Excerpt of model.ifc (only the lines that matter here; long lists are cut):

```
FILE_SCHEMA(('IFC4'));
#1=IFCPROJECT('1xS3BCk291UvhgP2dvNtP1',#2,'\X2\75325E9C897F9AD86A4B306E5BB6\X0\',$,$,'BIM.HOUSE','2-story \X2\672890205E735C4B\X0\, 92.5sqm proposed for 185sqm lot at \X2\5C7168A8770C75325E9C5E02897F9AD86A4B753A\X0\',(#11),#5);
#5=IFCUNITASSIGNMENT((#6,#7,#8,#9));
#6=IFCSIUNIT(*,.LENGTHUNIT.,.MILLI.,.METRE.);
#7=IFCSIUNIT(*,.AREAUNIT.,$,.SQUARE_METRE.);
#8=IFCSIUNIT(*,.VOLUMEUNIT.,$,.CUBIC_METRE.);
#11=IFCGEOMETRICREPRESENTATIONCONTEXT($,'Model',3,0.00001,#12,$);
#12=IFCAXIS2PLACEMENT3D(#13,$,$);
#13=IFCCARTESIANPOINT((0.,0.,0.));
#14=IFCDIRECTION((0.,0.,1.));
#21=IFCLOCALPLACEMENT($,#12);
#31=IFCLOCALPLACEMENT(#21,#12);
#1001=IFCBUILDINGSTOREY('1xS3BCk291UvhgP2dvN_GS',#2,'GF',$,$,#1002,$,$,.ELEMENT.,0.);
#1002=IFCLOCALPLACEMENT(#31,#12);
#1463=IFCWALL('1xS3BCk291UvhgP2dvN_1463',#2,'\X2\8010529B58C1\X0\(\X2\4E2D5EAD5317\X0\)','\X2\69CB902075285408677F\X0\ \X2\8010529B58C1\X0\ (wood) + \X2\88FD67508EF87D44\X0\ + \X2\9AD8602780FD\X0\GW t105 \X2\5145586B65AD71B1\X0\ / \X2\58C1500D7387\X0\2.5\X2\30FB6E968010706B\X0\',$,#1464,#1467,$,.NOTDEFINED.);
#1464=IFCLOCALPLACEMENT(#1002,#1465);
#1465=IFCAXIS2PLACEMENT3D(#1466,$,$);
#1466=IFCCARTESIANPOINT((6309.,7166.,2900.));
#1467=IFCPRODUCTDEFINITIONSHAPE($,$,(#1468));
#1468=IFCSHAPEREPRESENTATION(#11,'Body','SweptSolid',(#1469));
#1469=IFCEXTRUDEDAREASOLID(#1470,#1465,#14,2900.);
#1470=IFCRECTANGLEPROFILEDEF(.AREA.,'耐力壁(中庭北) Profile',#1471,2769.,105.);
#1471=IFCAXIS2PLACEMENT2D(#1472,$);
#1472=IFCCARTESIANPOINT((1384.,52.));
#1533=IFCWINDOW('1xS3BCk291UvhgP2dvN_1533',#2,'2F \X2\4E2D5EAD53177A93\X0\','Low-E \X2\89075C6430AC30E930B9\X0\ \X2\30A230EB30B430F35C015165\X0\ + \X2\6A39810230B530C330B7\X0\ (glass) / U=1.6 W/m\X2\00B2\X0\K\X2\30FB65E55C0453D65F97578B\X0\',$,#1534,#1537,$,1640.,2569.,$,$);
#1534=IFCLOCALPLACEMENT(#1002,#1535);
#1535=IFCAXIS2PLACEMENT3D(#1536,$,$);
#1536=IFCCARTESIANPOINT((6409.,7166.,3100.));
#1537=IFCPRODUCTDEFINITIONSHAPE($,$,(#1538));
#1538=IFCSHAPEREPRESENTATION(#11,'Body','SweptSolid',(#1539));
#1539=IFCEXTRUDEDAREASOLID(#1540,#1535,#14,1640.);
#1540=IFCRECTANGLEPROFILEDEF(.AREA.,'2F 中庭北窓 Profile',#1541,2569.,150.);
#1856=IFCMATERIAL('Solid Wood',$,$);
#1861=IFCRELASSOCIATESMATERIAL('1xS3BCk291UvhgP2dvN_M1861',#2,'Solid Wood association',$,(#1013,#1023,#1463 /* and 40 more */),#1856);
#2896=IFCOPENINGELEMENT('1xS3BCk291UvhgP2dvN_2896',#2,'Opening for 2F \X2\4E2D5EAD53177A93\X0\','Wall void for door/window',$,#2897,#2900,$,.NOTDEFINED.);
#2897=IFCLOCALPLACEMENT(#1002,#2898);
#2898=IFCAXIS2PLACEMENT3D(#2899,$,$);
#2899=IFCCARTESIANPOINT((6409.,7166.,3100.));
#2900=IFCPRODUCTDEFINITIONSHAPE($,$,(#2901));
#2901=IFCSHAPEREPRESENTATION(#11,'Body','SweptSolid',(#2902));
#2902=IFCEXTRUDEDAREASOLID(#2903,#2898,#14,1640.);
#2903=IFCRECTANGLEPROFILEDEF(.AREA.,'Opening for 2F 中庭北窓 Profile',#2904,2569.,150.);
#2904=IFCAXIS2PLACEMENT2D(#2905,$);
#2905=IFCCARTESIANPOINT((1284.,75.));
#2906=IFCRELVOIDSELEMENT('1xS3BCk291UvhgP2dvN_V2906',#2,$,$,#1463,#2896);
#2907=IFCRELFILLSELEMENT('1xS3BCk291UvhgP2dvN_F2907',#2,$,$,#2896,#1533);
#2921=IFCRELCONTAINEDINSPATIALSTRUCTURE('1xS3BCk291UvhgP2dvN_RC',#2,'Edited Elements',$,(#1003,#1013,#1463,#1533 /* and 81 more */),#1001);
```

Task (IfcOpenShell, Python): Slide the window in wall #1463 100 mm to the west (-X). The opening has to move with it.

```python
import ifcopenshell
import ifcopenshell.api.geometry
import ifcopenshell.util.placement

model = ifcopenshell.open("model.ifc")

window = model.by_guid("1xS3BCk291UvhgP2dvN_1533")
opening = window.FillsVoids[0].RelatingOpeningElement
wall = opening.VoidsElements[0].RelatingBuildingElement

wall_matrix = ifcopenshell.util.placement.get_local_placement(wall.ObjectPlacement)
shift = wall_matrix[:3, 0] * -100.0
before = ifcopenshell.util.placement.get_local_placement(window.ObjectPlacement)[:3, 3].copy()

# The window is not placed relative to its opening, so move both.
for product in (opening, window):
    matrix = ifcopenshell.util.placement.get_local_placement(product.ObjectPlacement)
    matrix[:3, 3] += shift
    ifcopenshell.api.geometry.edit_object_placement(model, product=product, matrix=matrix, is_si=False)

after = ifcopenshell.util.placement.get_local_placement(window.ObjectPlacement)[:3, 3]
print("window moved by", (after - before).round(3) + 0.0)

model.write("model_edited.ifc")
```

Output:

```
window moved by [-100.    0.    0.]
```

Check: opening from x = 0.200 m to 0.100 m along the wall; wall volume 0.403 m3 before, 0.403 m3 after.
